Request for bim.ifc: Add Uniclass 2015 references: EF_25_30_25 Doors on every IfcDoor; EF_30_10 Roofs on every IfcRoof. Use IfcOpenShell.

First a look at what the model holds.

```python
import ifcopenshell

model = ifcopenshell.open("bim.ifc")
print(model.schema)
print("classifications:", [c.Name for c in model.by_type("IfcClassification")])
for ifc_class in ("IfcDoor", "IfcRoof", "IfcStair", "IfcWall", "IfcWindow"):
    print(ifc_class, len(model.by_type(ifc_class)))
```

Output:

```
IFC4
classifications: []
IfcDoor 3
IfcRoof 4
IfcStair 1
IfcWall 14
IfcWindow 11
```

```python
import ifcopenshell
import ifcopenshell.api.classification

model = ifcopenshell.open("bim.ifc")

system = ifcopenshell.api.classification.add_classification(model, classification="Uniclass 2015")

codes = {
    "IfcDoor": ("EF_25_30_25", "Doors"),
    "IfcRoof": ("EF_30_10", "Roofs"),
}
for ifc_class, (code, name) in codes.items():
    products = model.by_type(ifc_class)
    ifcopenshell.api.classification.add_reference(
        model, products=products, classification=system, identification=code, name=name
    )
    print(code, len(products))

model.write("bim-out.ifc")
```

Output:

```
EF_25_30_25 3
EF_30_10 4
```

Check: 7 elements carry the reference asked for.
